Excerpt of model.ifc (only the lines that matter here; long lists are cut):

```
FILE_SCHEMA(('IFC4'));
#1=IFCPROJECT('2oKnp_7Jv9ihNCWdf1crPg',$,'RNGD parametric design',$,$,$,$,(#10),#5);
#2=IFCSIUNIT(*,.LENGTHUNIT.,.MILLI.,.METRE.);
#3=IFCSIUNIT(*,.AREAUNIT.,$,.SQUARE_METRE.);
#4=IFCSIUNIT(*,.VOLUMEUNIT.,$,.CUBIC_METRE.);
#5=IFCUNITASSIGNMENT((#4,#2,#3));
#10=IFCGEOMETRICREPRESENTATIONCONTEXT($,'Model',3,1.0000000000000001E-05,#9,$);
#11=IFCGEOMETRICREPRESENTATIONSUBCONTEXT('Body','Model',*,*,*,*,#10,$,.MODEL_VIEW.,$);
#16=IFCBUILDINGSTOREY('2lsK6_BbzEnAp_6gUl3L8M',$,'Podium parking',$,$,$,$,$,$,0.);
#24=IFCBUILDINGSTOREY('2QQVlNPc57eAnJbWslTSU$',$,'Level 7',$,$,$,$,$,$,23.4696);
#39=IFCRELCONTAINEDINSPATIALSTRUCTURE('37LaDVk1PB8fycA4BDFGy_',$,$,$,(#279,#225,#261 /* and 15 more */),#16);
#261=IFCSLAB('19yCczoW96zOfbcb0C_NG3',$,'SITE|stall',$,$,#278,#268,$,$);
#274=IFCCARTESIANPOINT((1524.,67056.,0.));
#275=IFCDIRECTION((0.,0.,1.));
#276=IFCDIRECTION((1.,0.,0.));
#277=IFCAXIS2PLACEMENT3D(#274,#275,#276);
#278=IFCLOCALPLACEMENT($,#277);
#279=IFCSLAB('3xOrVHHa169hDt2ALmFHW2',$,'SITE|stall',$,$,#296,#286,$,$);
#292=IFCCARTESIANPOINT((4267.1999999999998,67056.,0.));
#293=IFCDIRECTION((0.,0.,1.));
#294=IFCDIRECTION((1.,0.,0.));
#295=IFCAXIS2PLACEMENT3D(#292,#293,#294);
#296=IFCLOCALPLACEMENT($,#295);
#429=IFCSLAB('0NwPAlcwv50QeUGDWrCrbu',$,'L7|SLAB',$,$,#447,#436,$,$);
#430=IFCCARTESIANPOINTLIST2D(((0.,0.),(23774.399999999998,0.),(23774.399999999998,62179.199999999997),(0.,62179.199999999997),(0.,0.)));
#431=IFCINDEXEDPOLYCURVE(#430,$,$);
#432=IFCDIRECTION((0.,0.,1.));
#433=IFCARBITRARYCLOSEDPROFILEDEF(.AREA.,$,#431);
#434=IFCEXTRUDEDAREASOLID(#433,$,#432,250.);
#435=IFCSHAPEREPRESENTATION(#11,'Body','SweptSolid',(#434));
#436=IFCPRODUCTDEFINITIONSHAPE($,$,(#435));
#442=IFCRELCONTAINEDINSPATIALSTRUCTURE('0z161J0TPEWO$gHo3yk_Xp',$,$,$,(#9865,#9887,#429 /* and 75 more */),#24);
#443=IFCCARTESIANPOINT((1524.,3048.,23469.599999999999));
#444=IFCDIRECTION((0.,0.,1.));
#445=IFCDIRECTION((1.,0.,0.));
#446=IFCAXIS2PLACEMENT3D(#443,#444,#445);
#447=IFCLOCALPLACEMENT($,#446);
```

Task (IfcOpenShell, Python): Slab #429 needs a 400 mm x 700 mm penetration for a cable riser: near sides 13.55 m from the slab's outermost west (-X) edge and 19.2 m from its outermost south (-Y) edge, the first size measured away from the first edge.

```python
import numpy as np
import ifcopenshell
import ifcopenshell.api.feature
import ifcopenshell.api.geometry
import ifcopenshell.api.root
import ifcopenshell.geom
import ifcopenshell.util.placement
import ifcopenshell.util.representation
import ifcopenshell.util.shape
import ifcopenshell.util.unit

model = ifcopenshell.open("model.ifc")
unit_scale = ifcopenshell.util.unit.calculate_unit_scale(model)
settings = ifcopenshell.geom.settings()


def volume(element):
    """Net volume in cubic metres, openings subtracted."""
    shape = ifcopenshell.geom.create_shape(settings, element)
    return ifcopenshell.util.shape.get_volume(shape.geometry)


slab = model.by_guid("0NwPAlcwv50QeUGDWrCrbu")
before = volume(slab)

# Extent in the slab's own axes, in metres. The edges named are its -X and -Y sides.
slab_shape = ifcopenshell.geom.create_shape(settings, slab)
vertices = ifcopenshell.util.shape.get_vertices(slab_shape.geometry)
x_min, y_min, bottom = vertices.min(axis=0)
top = vertices[:, 2].max()

opening = ifcopenshell.api.root.create_entity(model, ifc_class="IfcOpeningElement", name="Cable riser opening", predefined_type="OPENING")
context = ifcopenshell.util.representation.get_context(model, "Model", "Body", "MODEL_VIEW")
width, depth = 0.4, 0.7
outline = [(0.0, 0.0), (width, 0.0), (width, depth), (0.0, depth), (0.0, 0.0)]
# Overshoot both faces by 50 mm so the cut is clean.
shape = ifcopenshell.api.geometry.add_slab_representation(
    model, context=context, depth=top - bottom + 0.1, polyline=outline
)
ifcopenshell.api.geometry.assign_representation(model, product=opening, representation=shape)

matrix = ifcopenshell.util.placement.get_local_placement(slab.ObjectPlacement)
matrix[:, 3] = matrix @ np.append(np.array([x_min + 13.55, y_min + 19.2, bottom - 0.05]) / unit_scale, 1.0)
ifcopenshell.api.geometry.edit_object_placement(model, product=opening, matrix=matrix, is_si=False)
ifcopenshell.api.feature.add_feature(model, feature=opening, element=slab)

after = volume(slab)

print(f"slab volume {before:.3f} -> {after:.3f} m3")

model.write("model_updated.ifc")
```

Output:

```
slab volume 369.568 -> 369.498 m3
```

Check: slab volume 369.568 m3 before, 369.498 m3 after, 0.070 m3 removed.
